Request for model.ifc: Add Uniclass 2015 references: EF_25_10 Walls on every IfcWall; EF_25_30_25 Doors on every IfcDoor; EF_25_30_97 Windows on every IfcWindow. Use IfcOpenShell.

First a look at what the model holds.

```python
import ifcopenshell

model = ifcopenshell.open("model.ifc")
print(model.schema)
print("classifications:", [c.Name for c in model.by_type("IfcClassification")])
for ifc_class in ("IfcDoor", "IfcRoof", "IfcStair", "IfcWall", "IfcWindow"):
    print(ifc_class, len(model.by_type(ifc_class)))
```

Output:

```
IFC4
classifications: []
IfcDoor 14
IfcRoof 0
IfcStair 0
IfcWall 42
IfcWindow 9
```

```python
import ifcopenshell
import ifcopenshell.api.classification

model = ifcopenshell.open("model.ifc")

system = ifcopenshell.api.classification.add_classification(model, classification="Uniclass 2015")

codes = {
    "IfcWall": ("EF_25_10", "Walls"),
    "IfcDoor": ("EF_25_30_25", "Doors"),
    "IfcWindow": ("EF_25_30_97", "Windows"),
}
for ifc_class, (code, name) in codes.items():
    products = model.by_type(ifc_class)
    ifcopenshell.api.classification.add_reference(
        model, products=products, classification=system, identification=code, name=name
    )
    print(code, len(products))

model.write("model-out.ifc")
```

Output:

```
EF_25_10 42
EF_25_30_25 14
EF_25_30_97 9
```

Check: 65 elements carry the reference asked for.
